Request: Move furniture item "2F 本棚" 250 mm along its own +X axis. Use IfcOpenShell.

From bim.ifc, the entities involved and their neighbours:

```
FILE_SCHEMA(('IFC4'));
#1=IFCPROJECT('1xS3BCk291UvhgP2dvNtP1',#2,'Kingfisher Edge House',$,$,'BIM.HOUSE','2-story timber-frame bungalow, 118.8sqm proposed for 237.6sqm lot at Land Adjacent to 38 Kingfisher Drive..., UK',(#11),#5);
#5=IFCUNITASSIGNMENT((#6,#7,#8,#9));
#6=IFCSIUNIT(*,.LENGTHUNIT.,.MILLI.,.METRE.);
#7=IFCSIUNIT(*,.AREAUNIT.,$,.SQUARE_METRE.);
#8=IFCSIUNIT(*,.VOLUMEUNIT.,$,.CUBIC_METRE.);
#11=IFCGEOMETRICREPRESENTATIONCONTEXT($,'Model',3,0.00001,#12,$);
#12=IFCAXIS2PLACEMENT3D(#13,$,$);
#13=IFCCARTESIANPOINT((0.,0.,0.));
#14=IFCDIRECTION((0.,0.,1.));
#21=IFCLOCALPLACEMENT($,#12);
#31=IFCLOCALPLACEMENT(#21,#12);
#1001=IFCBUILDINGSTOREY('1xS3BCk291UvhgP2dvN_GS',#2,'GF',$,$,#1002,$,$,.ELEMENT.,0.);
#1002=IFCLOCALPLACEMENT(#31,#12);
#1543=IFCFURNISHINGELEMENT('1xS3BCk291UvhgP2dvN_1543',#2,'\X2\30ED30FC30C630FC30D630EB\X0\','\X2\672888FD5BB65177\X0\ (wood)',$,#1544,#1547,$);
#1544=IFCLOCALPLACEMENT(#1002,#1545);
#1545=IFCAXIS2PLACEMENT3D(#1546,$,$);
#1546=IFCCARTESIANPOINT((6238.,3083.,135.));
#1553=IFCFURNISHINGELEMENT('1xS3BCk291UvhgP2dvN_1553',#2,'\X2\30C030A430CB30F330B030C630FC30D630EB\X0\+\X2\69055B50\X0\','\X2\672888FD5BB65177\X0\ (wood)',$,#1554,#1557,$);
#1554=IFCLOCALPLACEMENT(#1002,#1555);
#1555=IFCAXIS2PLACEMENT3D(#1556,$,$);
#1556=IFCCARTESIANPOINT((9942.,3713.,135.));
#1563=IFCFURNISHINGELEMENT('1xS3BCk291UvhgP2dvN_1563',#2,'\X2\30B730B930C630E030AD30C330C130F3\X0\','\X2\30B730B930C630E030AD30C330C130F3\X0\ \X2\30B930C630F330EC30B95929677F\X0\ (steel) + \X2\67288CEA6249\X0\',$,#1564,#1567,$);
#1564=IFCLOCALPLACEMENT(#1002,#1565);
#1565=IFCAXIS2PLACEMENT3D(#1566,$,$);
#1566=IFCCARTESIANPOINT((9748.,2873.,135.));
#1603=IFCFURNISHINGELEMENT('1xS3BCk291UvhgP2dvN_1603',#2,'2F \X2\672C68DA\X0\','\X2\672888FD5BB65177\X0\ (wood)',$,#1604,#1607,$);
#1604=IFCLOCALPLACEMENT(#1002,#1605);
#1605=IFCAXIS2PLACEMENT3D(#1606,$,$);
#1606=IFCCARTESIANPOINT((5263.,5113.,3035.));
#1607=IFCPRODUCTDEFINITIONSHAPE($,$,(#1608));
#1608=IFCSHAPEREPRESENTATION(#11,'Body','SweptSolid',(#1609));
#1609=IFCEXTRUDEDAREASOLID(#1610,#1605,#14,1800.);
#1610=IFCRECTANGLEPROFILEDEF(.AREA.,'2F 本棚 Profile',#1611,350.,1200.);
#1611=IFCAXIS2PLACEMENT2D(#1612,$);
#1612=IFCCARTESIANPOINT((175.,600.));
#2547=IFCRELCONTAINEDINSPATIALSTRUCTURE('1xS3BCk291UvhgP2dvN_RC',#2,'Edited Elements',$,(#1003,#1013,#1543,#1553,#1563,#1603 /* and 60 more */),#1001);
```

```python
import ifcopenshell
import ifcopenshell.api.geometry
import ifcopenshell.util.placement

model = ifcopenshell.open("bim.ifc")

item = model.by_guid("1xS3BCk291UvhgP2dvN_1603")
matrix = ifcopenshell.util.placement.get_local_placement(item.ObjectPlacement)
matrix[:3, 3] += matrix[:3, 0] * 250.0
ifcopenshell.api.geometry.edit_object_placement(model, product=item, matrix=matrix, is_si=False)

print(ifcopenshell.util.placement.get_local_placement(item.ObjectPlacement).round(3) + 0.0)

model.write("bim_edited.ifc")
```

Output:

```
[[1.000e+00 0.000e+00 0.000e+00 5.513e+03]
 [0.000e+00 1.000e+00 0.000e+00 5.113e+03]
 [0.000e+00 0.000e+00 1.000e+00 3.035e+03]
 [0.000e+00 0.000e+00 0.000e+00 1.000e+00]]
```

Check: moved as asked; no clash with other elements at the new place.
